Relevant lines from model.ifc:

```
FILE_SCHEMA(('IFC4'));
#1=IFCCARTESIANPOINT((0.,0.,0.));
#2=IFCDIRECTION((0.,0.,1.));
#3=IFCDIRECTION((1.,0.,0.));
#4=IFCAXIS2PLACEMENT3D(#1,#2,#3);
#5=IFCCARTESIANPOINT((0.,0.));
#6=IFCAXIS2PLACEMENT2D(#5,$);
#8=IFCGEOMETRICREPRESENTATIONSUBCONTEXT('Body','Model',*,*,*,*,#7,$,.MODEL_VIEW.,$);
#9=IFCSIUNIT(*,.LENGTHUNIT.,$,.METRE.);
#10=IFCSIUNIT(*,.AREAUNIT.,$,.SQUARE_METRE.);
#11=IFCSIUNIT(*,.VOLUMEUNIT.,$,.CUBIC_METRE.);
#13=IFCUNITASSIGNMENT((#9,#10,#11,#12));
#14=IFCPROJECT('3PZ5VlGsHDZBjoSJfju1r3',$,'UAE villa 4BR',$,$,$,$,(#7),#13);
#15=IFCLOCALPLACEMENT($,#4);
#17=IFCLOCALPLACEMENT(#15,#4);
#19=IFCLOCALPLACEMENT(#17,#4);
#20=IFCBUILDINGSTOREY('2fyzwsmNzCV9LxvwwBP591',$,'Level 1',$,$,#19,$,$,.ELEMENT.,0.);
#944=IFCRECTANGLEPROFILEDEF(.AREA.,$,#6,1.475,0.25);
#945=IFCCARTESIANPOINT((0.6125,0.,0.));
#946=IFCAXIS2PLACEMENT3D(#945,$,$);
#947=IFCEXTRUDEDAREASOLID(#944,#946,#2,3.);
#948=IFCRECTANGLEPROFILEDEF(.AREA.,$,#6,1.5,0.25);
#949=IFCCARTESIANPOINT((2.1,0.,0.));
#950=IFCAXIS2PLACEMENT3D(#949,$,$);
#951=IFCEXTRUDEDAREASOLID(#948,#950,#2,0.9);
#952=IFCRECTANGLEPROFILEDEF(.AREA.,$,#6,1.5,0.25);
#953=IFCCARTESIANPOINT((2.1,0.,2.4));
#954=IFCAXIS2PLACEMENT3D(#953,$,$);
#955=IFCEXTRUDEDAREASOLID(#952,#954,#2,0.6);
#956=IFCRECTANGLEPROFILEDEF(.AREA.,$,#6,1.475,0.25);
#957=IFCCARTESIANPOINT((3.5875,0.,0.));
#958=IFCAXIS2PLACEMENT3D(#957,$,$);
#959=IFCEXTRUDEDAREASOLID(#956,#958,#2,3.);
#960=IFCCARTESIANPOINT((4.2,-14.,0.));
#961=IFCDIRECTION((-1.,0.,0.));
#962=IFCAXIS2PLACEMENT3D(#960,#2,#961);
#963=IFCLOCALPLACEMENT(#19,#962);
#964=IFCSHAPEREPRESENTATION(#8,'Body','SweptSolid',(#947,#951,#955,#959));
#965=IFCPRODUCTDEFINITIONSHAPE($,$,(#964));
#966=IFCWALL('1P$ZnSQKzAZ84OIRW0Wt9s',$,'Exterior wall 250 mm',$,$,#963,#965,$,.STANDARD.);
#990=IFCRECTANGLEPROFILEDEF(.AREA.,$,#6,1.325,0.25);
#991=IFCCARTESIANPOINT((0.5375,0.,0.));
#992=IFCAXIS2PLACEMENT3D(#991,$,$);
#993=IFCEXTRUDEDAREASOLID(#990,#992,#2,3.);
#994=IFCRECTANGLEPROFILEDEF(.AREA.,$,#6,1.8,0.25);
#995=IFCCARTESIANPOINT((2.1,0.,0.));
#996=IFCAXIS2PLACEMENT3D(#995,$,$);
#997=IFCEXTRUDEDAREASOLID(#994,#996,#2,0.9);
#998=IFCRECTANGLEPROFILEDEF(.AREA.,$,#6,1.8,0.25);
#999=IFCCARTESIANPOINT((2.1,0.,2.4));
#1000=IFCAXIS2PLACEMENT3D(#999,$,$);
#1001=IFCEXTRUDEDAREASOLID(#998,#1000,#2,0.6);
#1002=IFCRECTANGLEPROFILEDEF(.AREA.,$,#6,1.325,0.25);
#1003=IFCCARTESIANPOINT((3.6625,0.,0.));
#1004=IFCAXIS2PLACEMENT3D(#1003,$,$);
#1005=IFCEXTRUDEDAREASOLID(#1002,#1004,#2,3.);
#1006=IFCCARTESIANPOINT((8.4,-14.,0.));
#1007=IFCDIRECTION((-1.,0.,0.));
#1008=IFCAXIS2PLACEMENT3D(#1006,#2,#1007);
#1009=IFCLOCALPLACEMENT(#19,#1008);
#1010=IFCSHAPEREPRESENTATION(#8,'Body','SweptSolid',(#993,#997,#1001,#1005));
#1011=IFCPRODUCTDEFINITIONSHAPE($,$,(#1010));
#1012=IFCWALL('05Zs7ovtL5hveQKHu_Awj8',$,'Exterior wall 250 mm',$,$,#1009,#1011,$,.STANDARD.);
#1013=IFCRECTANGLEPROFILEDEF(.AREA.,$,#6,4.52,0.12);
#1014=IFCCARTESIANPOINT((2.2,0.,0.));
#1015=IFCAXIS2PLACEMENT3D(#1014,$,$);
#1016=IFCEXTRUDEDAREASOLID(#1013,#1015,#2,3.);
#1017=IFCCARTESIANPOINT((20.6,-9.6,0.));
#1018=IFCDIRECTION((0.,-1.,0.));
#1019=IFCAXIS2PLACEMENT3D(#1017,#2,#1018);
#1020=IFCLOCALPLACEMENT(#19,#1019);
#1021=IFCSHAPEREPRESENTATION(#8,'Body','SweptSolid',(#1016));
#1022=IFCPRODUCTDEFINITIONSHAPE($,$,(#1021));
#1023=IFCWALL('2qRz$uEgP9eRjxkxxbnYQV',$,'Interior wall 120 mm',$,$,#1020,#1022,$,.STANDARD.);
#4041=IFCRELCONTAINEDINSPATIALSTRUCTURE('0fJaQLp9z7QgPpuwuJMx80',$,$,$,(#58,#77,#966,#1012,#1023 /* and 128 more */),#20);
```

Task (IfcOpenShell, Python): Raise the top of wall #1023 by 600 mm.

```python
import ifcopenshell
import ifcopenshell.geom
import ifcopenshell.util.representation
import ifcopenshell.util.shape

model = ifcopenshell.open("model.ifc")
settings = ifcopenshell.geom.settings()


def volume(element):
    """Net volume in cubic metres, openings subtracted."""
    shape = ifcopenshell.geom.create_shape(settings, element)
    return ifcopenshell.util.shape.get_volume(shape.geometry)


wall = model.by_guid("2qRz$uEgP9eRjxkxxbnYQV")
before = volume(wall)

body = ifcopenshell.util.representation.get_representation(wall, "Model", "Body")
solid = body.Items[0]
old_height = solid.Depth
solid.Depth += 0.6
after = volume(wall)

print(f"height {old_height:g} -> {solid.Depth:g}, volume {before:.3f} -> {after:.3f} m3")

model.write("model_edited.ifc")
```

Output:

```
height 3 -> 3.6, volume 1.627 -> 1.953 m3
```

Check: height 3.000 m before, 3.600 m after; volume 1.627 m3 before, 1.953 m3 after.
